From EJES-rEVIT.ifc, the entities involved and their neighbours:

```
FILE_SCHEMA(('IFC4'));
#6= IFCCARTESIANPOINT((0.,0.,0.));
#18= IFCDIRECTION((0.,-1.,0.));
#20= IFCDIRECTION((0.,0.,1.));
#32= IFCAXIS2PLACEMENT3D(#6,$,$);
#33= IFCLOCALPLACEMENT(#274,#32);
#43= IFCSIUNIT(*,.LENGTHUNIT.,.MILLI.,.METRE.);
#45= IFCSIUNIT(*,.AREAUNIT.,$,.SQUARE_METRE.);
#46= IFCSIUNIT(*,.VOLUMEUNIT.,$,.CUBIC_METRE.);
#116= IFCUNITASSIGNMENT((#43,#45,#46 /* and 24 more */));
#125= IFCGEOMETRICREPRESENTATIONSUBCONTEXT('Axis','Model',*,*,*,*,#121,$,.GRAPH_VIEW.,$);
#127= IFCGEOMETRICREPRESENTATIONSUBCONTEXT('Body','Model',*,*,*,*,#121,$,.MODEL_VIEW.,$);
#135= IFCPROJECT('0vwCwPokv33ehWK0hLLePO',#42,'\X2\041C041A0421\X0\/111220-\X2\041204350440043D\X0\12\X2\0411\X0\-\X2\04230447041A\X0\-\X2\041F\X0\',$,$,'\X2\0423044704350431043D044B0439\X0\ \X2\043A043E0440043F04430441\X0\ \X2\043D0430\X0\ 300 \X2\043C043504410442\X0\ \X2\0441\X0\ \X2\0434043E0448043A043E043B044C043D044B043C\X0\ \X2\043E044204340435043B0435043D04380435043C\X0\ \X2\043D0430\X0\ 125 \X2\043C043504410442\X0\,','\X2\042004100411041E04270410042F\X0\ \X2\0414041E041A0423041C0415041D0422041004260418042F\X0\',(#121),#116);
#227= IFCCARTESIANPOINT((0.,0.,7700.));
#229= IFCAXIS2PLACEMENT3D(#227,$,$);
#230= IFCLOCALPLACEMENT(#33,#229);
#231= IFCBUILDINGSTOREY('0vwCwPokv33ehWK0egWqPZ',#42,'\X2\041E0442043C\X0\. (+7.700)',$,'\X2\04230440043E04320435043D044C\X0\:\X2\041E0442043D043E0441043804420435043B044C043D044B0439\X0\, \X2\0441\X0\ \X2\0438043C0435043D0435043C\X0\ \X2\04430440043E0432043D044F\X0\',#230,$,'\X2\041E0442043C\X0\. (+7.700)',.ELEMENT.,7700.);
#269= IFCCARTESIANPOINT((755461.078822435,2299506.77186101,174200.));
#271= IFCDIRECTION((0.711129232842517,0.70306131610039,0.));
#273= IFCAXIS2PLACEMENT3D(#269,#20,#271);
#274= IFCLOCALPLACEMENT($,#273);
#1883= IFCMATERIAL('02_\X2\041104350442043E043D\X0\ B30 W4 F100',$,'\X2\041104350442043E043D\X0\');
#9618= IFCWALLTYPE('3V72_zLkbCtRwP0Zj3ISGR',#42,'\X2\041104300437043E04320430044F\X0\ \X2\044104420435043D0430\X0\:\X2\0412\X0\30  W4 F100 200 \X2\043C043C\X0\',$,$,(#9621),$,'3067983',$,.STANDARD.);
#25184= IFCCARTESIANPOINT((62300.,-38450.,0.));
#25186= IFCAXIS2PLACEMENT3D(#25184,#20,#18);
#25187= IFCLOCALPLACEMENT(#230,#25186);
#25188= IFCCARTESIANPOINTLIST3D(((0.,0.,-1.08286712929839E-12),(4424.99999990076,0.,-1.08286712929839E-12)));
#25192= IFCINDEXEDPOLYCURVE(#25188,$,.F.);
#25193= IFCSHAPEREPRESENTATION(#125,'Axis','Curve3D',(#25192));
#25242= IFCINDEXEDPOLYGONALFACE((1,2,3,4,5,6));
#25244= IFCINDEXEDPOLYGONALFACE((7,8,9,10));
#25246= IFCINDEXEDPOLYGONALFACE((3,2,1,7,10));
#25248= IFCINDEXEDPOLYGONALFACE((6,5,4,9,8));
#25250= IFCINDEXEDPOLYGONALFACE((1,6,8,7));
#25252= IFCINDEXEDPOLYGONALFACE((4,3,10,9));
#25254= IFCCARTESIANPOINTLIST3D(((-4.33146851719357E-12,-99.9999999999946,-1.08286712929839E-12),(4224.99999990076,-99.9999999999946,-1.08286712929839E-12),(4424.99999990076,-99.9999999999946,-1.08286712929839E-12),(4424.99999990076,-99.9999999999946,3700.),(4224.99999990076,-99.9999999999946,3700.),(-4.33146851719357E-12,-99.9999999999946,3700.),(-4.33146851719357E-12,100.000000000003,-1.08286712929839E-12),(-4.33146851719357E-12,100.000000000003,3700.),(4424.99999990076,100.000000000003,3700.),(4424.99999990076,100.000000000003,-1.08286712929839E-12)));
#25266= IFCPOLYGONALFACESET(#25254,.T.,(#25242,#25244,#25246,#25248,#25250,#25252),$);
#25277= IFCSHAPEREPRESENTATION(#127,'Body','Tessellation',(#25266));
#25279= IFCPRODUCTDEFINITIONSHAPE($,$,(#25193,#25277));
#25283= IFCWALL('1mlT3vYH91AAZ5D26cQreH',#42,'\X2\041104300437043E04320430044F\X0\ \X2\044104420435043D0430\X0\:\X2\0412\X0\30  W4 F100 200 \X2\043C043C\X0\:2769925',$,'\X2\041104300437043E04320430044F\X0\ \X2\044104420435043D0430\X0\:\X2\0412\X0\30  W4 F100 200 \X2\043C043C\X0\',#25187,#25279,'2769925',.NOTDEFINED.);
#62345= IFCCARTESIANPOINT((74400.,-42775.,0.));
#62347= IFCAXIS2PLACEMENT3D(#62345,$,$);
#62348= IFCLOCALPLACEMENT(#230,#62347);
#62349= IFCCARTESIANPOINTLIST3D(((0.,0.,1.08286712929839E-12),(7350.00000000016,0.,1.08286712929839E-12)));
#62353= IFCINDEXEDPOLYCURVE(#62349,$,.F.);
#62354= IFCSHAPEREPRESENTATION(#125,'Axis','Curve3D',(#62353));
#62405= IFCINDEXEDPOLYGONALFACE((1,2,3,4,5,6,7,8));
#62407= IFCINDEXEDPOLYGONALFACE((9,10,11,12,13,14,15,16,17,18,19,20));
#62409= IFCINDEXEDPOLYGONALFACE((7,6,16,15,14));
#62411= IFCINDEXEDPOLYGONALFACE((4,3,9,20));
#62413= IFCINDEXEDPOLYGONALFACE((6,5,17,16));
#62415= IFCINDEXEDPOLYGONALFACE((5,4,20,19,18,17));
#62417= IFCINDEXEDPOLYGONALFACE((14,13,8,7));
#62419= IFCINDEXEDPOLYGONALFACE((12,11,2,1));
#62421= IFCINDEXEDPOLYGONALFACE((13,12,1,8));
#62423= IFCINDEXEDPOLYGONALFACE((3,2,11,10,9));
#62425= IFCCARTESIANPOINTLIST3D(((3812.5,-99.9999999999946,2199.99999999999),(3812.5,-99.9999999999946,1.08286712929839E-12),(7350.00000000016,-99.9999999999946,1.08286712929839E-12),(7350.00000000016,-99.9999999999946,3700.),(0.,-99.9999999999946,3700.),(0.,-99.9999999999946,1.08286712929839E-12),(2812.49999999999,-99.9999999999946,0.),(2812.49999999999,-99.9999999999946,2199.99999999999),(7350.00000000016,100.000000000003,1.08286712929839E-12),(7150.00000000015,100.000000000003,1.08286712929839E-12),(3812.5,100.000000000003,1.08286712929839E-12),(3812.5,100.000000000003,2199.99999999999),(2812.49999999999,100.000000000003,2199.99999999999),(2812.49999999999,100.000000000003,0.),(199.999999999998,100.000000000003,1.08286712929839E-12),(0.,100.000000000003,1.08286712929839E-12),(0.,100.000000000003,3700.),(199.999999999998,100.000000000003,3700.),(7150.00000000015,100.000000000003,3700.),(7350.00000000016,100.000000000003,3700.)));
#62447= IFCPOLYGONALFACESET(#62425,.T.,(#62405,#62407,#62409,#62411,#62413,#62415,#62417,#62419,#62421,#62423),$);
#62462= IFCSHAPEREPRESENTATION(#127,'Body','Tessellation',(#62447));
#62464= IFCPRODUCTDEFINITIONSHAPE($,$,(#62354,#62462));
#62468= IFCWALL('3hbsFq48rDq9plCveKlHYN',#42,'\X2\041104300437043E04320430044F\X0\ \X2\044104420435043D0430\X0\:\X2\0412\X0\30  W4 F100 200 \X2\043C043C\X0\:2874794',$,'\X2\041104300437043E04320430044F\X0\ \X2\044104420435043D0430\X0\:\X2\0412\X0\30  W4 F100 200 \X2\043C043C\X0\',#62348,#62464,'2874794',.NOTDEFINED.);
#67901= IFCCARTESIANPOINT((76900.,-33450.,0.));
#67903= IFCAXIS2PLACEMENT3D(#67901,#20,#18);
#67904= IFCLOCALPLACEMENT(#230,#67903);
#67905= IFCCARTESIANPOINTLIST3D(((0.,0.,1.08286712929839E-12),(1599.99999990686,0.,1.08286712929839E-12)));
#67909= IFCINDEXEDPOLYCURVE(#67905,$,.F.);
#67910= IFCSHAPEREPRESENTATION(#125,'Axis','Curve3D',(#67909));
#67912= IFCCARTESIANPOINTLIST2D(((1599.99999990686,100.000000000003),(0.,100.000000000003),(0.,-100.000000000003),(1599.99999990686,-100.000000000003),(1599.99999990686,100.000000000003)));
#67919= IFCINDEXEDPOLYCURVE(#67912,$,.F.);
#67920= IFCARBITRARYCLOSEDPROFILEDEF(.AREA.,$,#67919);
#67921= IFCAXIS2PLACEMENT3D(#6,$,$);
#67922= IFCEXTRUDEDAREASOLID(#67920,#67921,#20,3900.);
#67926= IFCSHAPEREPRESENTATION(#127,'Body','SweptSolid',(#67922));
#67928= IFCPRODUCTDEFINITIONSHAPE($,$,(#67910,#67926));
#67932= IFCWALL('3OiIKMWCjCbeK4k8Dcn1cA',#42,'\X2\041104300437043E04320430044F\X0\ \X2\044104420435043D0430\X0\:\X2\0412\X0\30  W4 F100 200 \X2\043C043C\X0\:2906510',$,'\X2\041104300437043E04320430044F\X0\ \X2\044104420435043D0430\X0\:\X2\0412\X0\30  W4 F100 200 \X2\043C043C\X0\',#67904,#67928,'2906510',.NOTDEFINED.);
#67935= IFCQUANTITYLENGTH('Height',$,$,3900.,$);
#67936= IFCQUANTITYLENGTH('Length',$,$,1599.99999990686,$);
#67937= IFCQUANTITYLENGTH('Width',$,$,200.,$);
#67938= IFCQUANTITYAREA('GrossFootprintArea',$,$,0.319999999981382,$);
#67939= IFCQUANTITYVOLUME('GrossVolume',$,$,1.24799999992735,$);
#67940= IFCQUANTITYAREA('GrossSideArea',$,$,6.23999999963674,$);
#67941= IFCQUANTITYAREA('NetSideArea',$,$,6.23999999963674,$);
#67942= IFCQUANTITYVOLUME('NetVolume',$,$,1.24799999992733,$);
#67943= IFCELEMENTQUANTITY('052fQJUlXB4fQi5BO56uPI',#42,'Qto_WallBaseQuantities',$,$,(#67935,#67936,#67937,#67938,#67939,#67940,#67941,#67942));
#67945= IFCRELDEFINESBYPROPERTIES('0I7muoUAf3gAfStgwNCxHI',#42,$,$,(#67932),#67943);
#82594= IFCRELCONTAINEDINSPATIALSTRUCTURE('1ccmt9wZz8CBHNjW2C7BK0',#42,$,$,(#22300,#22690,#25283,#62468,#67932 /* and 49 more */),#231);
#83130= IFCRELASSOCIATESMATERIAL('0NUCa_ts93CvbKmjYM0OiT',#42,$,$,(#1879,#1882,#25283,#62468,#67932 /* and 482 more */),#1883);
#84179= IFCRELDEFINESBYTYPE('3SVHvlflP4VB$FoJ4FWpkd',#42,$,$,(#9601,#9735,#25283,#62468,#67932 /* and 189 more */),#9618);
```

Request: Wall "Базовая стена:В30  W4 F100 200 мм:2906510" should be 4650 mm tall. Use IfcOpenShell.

```python
import ifcopenshell
import ifcopenshell.api.pset
import ifcopenshell.geom
import ifcopenshell.util.element
import ifcopenshell.util.representation
import ifcopenshell.util.shape
import ifcopenshell.util.unit

model = ifcopenshell.open("EJES-rEVIT.ifc")
unit_scale = ifcopenshell.util.unit.calculate_unit_scale(model)
area_scale = ifcopenshell.util.unit.calculate_unit_scale(model, "AREAUNIT")
volume_scale = ifcopenshell.util.unit.calculate_unit_scale(model, "VOLUMEUNIT")
settings = ifcopenshell.geom.settings()


def volume(element):
    """Net volume in cubic metres, openings subtracted."""
    shape = ifcopenshell.geom.create_shape(settings, element)
    return ifcopenshell.util.shape.get_volume(shape.geometry)


wall = model.by_id(67932)
before = volume(wall)

body = ifcopenshell.util.representation.get_representation(wall, "Model", "Body")
solid = body.Items[0]
old_height = solid.Depth
solid.Depth = 4.65 / unit_scale
after = volume(wall)
thickness = 0.2  # wall thickness in metres

# Update the stored height, areas and volumes.
qto = model.by_id(ifcopenshell.util.element.get_pset(wall, "Qto_WallBaseQuantities", should_inherit=False)["id"])
ifcopenshell.api.pset.edit_qto(model, qto=qto, properties={
    "Height": solid.Depth,
    "GrossVolume": ifcopenshell.util.element.get_pset(wall, "Qto_WallBaseQuantities", "GrossVolume") * solid.Depth / old_height,
    "GrossSideArea": ifcopenshell.util.element.get_pset(wall, "Qto_WallBaseQuantities", "GrossSideArea") * solid.Depth / old_height,
    "NetSideArea": after / thickness / area_scale,
    "NetVolume": after / volume_scale,
})

print(f"height {old_height:g} -> {solid.Depth:g}, volume {before:.3f} -> {after:.3f} m3")

model.write("EJES-rEVIT_rev.ifc")
```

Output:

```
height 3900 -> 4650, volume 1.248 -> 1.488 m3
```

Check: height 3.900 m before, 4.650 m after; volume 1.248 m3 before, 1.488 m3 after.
